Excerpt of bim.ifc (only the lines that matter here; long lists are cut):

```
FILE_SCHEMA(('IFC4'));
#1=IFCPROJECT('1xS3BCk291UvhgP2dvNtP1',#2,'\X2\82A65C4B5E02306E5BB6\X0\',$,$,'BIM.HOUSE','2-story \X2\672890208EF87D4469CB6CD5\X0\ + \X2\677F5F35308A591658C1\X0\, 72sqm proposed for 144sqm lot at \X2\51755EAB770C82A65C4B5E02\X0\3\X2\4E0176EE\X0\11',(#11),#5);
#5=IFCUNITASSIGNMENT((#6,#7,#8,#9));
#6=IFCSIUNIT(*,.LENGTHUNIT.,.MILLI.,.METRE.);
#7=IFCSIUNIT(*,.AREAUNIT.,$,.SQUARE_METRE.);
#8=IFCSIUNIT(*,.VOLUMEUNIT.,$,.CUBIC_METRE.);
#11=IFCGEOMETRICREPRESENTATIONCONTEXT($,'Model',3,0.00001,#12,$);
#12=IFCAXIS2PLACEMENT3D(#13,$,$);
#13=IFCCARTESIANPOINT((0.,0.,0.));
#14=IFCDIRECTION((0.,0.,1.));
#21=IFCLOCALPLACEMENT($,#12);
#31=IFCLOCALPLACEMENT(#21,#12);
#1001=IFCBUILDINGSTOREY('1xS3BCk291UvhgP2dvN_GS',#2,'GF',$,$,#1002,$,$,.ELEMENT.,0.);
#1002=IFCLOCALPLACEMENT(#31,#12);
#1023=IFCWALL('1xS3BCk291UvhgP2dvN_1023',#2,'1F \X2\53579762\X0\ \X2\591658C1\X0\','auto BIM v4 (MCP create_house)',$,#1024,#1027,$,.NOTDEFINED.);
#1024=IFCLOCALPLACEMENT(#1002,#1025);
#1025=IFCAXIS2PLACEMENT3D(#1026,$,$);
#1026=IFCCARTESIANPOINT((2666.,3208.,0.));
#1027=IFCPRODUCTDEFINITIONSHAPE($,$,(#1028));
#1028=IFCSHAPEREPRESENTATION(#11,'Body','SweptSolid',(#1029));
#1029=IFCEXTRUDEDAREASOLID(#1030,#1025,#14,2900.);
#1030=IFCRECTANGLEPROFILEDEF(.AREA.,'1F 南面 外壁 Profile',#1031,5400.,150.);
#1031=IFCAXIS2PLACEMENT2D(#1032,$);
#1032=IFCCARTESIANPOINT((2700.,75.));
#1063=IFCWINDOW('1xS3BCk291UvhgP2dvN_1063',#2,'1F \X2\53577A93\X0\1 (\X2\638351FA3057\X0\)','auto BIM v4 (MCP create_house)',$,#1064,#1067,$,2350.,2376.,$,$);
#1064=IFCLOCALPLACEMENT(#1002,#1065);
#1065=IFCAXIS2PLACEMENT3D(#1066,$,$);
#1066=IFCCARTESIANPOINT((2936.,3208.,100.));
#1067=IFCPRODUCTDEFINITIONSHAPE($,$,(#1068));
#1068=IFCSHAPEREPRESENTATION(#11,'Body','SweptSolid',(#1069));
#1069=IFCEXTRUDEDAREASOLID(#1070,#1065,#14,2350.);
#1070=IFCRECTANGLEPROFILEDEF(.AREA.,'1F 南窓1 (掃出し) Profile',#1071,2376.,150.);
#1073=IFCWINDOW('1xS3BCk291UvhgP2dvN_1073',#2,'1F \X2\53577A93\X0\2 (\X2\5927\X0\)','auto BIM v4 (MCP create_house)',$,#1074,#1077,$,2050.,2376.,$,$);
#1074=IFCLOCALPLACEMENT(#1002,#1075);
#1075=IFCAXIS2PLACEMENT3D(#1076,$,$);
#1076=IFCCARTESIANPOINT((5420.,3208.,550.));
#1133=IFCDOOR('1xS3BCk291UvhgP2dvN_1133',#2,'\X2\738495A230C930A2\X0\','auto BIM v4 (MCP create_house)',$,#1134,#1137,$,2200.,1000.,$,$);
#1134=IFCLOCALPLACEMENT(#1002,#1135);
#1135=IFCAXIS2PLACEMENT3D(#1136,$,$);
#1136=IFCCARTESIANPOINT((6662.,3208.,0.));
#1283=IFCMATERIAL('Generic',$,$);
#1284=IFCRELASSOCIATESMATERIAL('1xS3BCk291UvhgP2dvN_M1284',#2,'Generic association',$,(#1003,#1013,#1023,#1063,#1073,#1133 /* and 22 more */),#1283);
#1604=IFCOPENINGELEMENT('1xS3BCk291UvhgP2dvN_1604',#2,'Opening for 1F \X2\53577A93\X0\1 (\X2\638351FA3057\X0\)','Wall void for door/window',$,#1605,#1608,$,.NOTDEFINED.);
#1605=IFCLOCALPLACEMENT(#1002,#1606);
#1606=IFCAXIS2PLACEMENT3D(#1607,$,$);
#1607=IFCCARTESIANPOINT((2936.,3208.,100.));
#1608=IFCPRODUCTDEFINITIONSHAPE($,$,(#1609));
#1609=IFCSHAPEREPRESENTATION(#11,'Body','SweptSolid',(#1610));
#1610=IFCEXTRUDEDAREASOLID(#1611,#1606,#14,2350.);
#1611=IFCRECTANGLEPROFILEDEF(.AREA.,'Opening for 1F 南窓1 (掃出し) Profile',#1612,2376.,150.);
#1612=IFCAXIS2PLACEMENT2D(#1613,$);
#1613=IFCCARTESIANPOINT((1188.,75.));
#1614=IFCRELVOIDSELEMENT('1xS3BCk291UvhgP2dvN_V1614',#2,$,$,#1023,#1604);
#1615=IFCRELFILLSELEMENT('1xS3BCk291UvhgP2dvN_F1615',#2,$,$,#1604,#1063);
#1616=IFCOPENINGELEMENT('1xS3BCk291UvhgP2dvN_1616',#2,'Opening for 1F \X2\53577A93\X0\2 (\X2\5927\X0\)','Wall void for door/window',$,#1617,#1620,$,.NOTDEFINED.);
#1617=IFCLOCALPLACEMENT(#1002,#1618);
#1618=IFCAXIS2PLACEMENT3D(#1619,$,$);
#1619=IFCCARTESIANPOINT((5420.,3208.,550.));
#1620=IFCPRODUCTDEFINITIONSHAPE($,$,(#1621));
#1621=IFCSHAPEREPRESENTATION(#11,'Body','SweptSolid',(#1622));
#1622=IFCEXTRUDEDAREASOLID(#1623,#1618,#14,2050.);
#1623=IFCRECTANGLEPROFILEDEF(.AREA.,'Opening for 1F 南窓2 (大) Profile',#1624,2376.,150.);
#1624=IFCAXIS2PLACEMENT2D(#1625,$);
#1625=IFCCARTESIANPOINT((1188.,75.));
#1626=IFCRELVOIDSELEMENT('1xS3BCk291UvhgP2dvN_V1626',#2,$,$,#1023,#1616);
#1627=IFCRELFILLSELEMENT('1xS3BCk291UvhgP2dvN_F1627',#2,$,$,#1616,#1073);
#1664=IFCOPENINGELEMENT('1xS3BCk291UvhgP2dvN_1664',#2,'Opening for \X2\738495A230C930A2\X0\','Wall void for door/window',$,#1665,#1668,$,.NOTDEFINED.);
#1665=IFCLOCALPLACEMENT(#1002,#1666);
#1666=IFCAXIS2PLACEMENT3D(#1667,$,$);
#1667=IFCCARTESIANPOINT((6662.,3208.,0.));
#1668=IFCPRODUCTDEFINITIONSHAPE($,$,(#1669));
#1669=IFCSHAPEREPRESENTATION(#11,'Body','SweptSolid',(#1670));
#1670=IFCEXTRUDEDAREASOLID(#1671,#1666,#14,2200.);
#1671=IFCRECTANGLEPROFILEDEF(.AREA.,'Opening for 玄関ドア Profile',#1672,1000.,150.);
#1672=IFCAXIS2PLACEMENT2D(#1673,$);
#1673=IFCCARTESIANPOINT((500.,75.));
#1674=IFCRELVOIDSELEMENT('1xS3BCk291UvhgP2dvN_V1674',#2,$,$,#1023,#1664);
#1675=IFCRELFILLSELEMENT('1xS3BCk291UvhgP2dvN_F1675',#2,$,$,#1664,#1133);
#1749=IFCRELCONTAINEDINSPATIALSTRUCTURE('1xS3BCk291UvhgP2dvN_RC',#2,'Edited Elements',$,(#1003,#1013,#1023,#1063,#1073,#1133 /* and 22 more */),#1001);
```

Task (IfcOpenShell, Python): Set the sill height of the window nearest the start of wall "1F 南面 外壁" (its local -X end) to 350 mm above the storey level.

```python
import numpy as np
import ifcopenshell
import ifcopenshell.api.geometry
import ifcopenshell.geom
import ifcopenshell.util.element
import ifcopenshell.util.placement
import ifcopenshell.util.shape
import ifcopenshell.util.unit

model = ifcopenshell.open("bim.ifc")
unit_scale = ifcopenshell.util.unit.calculate_unit_scale(model)

window = model.by_guid("1xS3BCk291UvhgP2dvN_1063")
opening = window.FillsVoids[0].RelatingOpeningElement
storey = ifcopenshell.util.element.get_container(window, ifc_class="IfcBuildingStorey")
level = ifcopenshell.util.placement.get_local_placement(storey.ObjectPlacement)[2, 3]

# The opening's origin need not be at the sill, so measure its lowest point.
shape = ifcopenshell.geom.create_shape(ifcopenshell.geom.settings(), opening)
bottom = ifcopenshell.util.shape.get_shape_bottom_elevation(shape, shape.geometry) / unit_scale
dz = level + 0.35 / unit_scale - bottom

shift = np.array([0.0, 0.0, dz])
# The window is not placed relative to its opening, so move both.
for product in (opening, window):
    matrix = ifcopenshell.util.placement.get_local_placement(product.ObjectPlacement)
    matrix[:3, 3] += shift
    ifcopenshell.api.geometry.edit_object_placement(model, product=product, matrix=matrix, is_si=False)

print(f"moved by {dz * unit_scale:+.3f} m")

model.write("bim_v2.ifc")
```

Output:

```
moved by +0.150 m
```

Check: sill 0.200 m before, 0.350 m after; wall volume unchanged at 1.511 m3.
